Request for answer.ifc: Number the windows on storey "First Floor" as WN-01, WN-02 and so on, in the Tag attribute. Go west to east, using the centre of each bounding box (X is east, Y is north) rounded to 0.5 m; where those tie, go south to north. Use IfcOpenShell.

First a look at what the model holds.

```python
import ifcopenshell
import ifcopenshell.util.element
import ifcopenshell.util.placement

model = ifcopenshell.open("answer.ifc")
print(model.schema)
storey = next(s for s in model.by_type("IfcBuildingStorey") if s.Name == "First Floor")
windows = [e for e in ifcopenshell.util.element.get_decomposition(storey) if e.is_a("IfcWindow")]
for e in sorted(windows, key=lambda e: e.id()):
    origin = ifcopenshell.util.placement.get_local_placement(e.ObjectPlacement)[:3, 3]
    print(e.id(), e.Tag, e.Name, origin.round(2) + 0.0, sep=" | ")
```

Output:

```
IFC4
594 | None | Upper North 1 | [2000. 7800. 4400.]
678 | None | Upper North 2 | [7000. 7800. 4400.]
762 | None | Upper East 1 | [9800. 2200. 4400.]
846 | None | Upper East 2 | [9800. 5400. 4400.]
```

```python
import ifcopenshell
import ifcopenshell.geom
import ifcopenshell.util.element
import ifcopenshell.util.shape

model = ifcopenshell.open("answer.ifc")
settings = ifcopenshell.geom.settings()
settings.set("use-world-coords", True)


def centre(element):
    shape = ifcopenshell.geom.create_shape(settings, element)
    return ifcopenshell.util.shape.get_bbox_centroid(shape.geometry)


storey = next(s for s in model.by_type("IfcBuildingStorey") if s.Name == "First Floor")
windows = [e for e in ifcopenshell.util.element.get_decomposition(storey) if e.is_a("IfcWindow")]

# Insertion points can sit at a corner or the storey origin, so sort by the geometry (in metres).
centres = {e: centre(e) for e in windows}
windows.sort(key=lambda e: (round(centres[e][0] / 0.5), centres[e][1]))

for i, e in enumerate(windows, start=1):
    number = f"WN-{i:02d}"
    e.Tag = number
    print(e.id(), number)

model.write("answer_updated.ifc")
```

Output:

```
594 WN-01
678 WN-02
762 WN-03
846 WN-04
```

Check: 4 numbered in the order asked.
